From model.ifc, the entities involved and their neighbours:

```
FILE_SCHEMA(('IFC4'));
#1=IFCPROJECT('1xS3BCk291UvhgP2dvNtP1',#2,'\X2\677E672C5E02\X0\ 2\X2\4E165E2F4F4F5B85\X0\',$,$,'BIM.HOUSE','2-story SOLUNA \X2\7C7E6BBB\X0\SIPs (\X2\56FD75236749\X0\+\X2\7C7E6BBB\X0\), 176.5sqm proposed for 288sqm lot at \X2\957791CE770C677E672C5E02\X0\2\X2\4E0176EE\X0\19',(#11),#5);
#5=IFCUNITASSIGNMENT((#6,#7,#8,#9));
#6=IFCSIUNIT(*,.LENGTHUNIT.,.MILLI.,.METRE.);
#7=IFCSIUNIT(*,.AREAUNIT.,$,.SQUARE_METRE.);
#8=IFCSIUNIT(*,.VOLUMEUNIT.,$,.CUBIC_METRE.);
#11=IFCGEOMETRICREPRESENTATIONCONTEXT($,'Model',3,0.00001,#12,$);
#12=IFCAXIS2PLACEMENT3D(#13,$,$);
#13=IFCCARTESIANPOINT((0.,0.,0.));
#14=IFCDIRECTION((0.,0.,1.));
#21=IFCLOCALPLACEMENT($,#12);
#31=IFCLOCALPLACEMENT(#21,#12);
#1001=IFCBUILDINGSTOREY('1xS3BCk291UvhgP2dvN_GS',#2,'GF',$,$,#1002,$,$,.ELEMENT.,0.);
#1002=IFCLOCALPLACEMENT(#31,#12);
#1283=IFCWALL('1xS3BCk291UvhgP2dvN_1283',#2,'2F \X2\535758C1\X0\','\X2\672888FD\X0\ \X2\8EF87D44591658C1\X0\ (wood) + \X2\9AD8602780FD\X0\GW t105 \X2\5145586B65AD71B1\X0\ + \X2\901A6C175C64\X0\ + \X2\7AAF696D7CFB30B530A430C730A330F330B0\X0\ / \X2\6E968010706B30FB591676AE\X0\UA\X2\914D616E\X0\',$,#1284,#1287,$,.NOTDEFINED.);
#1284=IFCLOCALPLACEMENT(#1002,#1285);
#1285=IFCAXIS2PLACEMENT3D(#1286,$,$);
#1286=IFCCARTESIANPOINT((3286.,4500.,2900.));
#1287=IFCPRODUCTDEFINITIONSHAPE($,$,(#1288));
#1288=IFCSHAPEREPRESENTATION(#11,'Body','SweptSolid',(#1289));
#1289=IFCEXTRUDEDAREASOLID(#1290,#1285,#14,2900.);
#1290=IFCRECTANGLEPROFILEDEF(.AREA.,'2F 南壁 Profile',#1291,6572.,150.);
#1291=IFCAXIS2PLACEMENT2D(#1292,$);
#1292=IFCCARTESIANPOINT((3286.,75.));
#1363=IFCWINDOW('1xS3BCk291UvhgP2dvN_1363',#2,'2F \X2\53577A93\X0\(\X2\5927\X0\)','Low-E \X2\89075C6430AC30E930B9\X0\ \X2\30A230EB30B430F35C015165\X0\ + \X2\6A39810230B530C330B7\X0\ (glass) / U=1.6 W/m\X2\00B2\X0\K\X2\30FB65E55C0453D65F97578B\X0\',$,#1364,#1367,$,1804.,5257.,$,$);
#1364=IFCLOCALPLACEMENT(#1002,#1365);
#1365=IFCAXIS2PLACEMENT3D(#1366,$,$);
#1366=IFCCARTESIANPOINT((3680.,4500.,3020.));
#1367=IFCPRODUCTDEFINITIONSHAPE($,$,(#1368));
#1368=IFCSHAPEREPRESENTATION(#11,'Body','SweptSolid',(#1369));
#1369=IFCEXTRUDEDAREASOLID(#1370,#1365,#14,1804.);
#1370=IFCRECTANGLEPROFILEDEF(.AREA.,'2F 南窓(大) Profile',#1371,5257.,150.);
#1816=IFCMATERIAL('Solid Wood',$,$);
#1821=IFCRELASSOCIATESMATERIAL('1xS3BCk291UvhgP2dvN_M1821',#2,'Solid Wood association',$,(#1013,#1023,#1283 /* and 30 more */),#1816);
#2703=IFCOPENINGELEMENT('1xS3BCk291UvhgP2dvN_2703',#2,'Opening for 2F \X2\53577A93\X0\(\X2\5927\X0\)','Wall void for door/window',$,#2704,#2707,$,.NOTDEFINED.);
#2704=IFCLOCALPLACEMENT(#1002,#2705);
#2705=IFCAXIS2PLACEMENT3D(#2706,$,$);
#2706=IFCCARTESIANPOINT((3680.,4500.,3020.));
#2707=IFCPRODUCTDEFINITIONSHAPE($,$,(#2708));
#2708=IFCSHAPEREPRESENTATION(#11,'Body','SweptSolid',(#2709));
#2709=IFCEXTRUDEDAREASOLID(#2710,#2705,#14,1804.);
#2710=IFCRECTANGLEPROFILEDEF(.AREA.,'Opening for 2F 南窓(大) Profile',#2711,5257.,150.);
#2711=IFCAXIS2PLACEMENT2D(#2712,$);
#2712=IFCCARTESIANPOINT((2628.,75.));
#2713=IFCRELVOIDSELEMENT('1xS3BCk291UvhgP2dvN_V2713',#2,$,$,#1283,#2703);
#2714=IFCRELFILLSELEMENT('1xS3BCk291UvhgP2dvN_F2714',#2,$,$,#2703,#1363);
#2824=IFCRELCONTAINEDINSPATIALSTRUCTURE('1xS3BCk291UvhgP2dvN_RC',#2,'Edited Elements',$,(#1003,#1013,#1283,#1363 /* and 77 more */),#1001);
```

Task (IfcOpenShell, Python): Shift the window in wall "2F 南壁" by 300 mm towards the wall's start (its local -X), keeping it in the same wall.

```python
import ifcopenshell
import ifcopenshell.api.geometry
import ifcopenshell.util.placement
import ifcopenshell.util.unit

model = ifcopenshell.open("model.ifc")
unit_scale = ifcopenshell.util.unit.calculate_unit_scale(model)

window = model.by_id(1363)
opening = window.FillsVoids[0].RelatingOpeningElement
wall = opening.VoidsElements[0].RelatingBuildingElement

wall_matrix = ifcopenshell.util.placement.get_local_placement(wall.ObjectPlacement)
shift = wall_matrix[:3, 0] * -0.3 / unit_scale
before = ifcopenshell.util.placement.get_local_placement(window.ObjectPlacement)[:3, 3].copy()

# The window is not placed relative to its opening, so move both.
for product in (opening, window):
    matrix = ifcopenshell.util.placement.get_local_placement(product.ObjectPlacement)
    matrix[:3, 3] += shift
    ifcopenshell.api.geometry.edit_object_placement(model, product=product, matrix=matrix, is_si=False)

after = ifcopenshell.util.placement.get_local_placement(window.ObjectPlacement)[:3, 3]
print("window moved by", (after - before).round(3) + 0.0)

model.write("model_rev.ifc")
```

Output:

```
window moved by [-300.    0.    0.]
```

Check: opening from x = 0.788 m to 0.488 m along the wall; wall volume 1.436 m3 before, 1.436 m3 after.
